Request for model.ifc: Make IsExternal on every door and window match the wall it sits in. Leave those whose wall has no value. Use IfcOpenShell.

First a look at what the model holds.

```python
import ifcopenshell
import ifcopenshell.util.element

model = ifcopenshell.open("model.ifc")
print(model.schema)
seen = {}
for e in model.by_type("IfcDoor") + model.by_type("IfcWindow"):
    if not e.FillsVoids:
        continue
    host = e.FillsVoids[0].RelatingOpeningElement.VoidsElements[0].RelatingBuildingElement
    own = ifcopenshell.util.element.get_pset(e, f"Pset_{e.is_a()[3:].removesuffix('StandardCase')}Common", "IsExternal")
    wall = ifcopenshell.util.element.get_pset(host, "Pset_WallCommon", "IsExternal")
    seen[e.is_a(), own, wall] = seen.get((e.is_a(), own, wall), 0) + 1
for (cls, own, wall), count in sorted(seen.items(), key=str):
    print(count, cls, "IsExternal:", own, "| host wall:", wall)
```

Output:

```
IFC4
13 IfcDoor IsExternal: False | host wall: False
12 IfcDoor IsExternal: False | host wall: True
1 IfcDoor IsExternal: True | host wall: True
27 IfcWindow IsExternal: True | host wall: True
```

```python
import ifcopenshell
import ifcopenshell.api.pset
import ifcopenshell.util.element

model = ifcopenshell.open("model.ifc")

count = 0
for ifc_class, pset_name in (("IfcDoor", "Pset_DoorCommon"), ("IfcWindow", "Pset_WindowCommon")):
    for e in model.by_type(ifc_class):
        if not e.FillsVoids:
            continue
        host = e.FillsVoids[0].RelatingOpeningElement.VoidsElements[0].RelatingBuildingElement
        external = ifcopenshell.util.element.get_pset(host, "Pset_WallCommon", "IsExternal")
        if external is None or ifcopenshell.util.element.get_pset(e, pset_name, "IsExternal") == external:
            continue
        pset = ifcopenshell.api.pset.add_pset(model, product=e, name=pset_name)
        ifcopenshell.api.pset.edit_pset(model, pset=pset, properties={"IsExternal": external})
        count += 1

print(count, "updated")

model.write("model_v2.ifc")
```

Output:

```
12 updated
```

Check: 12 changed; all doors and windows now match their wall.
